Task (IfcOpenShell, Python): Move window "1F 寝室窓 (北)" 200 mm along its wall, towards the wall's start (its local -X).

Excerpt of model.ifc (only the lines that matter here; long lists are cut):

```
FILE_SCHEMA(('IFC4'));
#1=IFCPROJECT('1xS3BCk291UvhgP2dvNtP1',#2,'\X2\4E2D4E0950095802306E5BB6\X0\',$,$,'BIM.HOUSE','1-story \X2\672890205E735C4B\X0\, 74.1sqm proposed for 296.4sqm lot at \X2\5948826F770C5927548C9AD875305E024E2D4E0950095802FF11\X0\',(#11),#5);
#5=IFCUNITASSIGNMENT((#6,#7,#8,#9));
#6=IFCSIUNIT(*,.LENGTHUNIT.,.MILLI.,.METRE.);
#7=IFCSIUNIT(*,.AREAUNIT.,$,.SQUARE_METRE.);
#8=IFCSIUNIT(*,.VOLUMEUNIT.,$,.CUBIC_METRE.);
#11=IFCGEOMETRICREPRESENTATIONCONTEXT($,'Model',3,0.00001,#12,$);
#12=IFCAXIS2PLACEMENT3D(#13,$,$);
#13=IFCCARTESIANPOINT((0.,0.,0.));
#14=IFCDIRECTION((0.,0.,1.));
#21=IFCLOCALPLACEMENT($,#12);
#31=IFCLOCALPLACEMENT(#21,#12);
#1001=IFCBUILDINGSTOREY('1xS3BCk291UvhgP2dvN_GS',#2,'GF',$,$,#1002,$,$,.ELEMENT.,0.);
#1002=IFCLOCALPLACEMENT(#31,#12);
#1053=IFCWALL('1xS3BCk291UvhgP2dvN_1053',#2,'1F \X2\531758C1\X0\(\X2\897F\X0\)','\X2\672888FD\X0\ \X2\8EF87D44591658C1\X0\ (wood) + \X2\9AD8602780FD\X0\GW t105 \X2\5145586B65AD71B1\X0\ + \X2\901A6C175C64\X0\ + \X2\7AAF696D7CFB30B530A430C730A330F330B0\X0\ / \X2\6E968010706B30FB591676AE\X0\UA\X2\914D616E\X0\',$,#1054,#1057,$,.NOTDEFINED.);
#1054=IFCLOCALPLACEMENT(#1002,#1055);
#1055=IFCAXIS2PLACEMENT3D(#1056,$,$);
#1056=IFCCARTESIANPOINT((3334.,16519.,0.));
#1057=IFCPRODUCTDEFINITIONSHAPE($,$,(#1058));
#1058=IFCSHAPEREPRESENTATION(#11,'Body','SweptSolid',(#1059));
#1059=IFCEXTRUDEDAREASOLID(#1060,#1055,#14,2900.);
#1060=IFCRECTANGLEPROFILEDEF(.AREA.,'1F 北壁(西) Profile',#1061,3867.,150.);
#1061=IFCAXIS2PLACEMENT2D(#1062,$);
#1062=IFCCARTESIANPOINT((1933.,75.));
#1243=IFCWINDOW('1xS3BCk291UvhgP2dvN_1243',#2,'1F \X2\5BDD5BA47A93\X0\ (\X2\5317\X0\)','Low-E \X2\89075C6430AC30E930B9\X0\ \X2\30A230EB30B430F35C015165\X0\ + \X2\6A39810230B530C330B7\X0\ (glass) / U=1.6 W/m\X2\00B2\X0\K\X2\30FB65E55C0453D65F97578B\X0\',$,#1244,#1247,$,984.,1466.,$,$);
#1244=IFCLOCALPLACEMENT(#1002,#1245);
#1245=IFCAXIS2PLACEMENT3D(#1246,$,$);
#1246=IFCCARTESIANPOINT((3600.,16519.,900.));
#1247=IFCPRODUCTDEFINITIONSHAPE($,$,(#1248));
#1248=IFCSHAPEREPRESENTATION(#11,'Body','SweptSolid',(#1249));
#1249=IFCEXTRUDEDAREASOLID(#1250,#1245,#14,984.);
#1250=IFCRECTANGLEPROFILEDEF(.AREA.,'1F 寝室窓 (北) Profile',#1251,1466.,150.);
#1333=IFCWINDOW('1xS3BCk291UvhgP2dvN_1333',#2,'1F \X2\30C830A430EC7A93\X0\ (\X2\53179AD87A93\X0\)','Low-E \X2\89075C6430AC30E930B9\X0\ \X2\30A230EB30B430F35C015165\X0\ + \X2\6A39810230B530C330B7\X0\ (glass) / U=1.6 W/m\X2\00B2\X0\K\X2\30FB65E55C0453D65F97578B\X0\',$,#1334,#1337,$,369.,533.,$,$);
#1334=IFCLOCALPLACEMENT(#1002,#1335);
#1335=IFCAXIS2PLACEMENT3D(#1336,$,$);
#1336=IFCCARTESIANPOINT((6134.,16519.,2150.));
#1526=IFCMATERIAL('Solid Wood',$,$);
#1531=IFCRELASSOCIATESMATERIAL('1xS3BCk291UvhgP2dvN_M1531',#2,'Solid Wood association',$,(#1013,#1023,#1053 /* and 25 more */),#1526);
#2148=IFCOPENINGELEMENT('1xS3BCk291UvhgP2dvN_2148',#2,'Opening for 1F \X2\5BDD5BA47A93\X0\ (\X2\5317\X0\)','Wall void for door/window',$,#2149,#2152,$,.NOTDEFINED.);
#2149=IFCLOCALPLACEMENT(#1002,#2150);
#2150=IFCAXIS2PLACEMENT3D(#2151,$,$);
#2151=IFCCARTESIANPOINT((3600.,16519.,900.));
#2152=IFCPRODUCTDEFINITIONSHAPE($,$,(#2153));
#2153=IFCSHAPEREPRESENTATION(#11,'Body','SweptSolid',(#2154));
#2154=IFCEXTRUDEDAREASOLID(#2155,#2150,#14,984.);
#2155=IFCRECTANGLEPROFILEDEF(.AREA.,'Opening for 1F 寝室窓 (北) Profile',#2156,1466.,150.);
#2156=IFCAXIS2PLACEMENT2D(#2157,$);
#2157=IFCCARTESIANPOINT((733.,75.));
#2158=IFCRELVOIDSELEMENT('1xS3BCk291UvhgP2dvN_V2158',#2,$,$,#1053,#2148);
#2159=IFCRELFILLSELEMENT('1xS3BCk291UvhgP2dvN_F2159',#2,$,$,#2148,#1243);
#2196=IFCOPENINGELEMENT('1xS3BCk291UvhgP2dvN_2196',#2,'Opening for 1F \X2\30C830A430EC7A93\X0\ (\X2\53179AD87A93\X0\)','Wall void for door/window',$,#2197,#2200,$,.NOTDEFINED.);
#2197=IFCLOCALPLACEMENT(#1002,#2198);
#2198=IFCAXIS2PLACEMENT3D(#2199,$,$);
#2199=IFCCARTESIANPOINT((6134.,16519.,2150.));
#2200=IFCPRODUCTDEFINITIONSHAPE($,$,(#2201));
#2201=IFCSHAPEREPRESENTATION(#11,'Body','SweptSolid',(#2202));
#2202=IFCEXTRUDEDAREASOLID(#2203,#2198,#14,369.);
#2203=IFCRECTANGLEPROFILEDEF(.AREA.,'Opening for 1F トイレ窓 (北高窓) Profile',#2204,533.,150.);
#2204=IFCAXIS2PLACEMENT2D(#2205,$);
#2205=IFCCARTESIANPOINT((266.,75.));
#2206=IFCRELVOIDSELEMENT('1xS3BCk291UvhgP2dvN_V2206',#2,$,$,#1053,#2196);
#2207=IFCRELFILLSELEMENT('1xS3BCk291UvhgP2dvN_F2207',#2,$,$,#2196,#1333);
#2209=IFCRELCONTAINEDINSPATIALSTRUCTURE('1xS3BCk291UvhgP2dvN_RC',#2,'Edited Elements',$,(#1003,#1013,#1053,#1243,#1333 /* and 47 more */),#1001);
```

```python
import ifcopenshell
import ifcopenshell.api.geometry
import ifcopenshell.util.placement
import ifcopenshell.util.unit

model = ifcopenshell.open("model.ifc")
unit_scale = ifcopenshell.util.unit.calculate_unit_scale(model)

window = model.by_guid("1xS3BCk291UvhgP2dvN_1243")
opening = window.FillsVoids[0].RelatingOpeningElement
wall = opening.VoidsElements[0].RelatingBuildingElement

wall_matrix = ifcopenshell.util.placement.get_local_placement(wall.ObjectPlacement)
shift = wall_matrix[:3, 0] * -0.2 / unit_scale
before = ifcopenshell.util.placement.get_local_placement(window.ObjectPlacement)[:3, 3].copy()

# The window is not placed relative to its opening, so move both.
for product in (opening, window):
    matrix = ifcopenshell.util.placement.get_local_placement(product.ObjectPlacement)
    matrix[:3, 3] += shift
    ifcopenshell.api.geometry.edit_object_placement(model, product=product, matrix=matrix, is_si=False)

after = ifcopenshell.util.placement.get_local_placement(window.ObjectPlacement)[:3, 3]
print("window moved by", (after - before).round(3) + 0.0)

model.write("model_updated.ifc")
```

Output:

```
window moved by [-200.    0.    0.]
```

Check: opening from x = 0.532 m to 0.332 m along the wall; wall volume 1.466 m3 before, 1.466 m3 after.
